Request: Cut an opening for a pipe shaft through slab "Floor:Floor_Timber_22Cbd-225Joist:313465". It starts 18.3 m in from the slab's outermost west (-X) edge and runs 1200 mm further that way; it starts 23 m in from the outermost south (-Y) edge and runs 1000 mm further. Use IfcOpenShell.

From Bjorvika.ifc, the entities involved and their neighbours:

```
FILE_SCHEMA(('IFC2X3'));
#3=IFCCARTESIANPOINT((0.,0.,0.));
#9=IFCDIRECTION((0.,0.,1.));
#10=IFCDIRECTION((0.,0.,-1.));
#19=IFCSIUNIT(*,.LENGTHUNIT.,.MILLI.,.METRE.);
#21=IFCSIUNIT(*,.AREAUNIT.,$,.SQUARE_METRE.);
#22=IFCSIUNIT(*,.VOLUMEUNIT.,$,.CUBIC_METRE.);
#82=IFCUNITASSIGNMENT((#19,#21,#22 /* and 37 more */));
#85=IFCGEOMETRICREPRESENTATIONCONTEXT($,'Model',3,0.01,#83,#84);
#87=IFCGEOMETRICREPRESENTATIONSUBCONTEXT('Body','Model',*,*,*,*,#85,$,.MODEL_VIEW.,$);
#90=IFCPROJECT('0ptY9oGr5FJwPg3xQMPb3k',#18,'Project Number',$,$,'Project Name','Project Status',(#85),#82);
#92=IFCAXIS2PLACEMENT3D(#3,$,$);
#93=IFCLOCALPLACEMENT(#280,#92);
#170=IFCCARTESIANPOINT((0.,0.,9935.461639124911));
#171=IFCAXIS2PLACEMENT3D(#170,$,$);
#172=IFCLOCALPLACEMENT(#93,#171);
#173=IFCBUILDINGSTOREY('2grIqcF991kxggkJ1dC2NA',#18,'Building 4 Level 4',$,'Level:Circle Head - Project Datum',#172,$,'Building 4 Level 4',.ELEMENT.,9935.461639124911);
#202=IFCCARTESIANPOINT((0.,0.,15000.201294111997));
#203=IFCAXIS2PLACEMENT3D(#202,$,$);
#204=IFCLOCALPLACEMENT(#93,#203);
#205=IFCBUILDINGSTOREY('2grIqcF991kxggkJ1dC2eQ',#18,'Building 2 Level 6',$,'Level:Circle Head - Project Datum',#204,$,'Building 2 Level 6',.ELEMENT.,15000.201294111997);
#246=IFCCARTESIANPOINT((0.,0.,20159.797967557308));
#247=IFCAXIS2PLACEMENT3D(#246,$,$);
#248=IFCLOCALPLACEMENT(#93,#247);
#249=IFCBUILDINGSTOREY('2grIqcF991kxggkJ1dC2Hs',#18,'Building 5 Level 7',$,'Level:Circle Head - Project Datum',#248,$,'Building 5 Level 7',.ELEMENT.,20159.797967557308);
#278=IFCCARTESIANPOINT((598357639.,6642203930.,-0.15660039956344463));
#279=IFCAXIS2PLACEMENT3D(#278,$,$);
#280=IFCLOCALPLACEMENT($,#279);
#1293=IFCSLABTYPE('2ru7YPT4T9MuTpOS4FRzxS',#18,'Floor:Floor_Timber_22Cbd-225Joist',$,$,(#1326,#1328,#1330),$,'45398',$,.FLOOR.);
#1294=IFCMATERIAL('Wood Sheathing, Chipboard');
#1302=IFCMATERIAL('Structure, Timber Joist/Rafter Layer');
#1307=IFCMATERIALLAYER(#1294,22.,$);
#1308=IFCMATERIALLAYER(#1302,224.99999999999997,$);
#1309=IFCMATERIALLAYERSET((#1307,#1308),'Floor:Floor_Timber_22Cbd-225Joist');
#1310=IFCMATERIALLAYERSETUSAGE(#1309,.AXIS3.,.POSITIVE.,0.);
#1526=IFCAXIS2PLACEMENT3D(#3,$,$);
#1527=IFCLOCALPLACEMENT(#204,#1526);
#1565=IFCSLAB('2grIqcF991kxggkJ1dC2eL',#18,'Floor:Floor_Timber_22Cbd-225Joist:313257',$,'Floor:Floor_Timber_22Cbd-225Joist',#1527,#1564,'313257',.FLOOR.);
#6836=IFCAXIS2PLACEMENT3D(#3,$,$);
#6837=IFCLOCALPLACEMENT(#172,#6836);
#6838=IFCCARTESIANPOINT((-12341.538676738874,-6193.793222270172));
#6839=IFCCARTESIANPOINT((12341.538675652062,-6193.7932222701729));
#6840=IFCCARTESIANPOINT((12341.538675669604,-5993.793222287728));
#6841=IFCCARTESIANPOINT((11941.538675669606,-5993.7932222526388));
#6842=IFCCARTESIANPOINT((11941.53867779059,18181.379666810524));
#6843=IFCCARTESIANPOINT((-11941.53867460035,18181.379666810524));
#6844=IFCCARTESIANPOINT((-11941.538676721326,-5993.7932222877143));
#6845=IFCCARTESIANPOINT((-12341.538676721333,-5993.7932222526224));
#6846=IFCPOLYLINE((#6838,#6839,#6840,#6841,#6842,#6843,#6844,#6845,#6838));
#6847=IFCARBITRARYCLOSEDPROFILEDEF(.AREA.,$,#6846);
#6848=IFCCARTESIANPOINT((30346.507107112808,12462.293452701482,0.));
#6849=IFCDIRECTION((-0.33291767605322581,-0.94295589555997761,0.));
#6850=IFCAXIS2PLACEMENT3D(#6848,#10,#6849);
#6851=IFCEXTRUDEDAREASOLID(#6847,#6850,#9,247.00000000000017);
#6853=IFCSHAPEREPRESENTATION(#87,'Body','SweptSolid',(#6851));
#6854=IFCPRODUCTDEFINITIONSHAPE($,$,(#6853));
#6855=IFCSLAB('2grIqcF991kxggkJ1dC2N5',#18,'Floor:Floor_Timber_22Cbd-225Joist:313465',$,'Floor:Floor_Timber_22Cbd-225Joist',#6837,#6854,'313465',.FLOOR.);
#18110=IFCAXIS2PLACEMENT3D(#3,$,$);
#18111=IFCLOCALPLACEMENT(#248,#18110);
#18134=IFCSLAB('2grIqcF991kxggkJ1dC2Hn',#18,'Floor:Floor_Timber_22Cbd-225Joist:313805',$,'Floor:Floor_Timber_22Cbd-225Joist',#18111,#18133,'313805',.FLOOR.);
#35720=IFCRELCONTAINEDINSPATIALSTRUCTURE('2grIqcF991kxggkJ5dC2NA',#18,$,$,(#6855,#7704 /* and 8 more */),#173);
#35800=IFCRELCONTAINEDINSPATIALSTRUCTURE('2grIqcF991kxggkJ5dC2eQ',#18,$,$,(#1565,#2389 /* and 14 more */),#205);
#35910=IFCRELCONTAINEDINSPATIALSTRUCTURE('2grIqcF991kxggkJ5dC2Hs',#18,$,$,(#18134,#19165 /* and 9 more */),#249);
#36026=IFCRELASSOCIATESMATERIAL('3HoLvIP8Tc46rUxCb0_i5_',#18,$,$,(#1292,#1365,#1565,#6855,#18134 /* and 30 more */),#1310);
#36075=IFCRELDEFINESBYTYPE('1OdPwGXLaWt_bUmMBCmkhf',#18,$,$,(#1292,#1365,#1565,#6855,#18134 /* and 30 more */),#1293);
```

```python
import numpy as np
import ifcopenshell
import ifcopenshell.api.feature
import ifcopenshell.api.geometry
import ifcopenshell.api.root
import ifcopenshell.geom
import ifcopenshell.util.placement
import ifcopenshell.util.representation
import ifcopenshell.util.shape
import ifcopenshell.util.unit

model = ifcopenshell.open("Bjorvika.ifc")
unit_scale = ifcopenshell.util.unit.calculate_unit_scale(model)
settings = ifcopenshell.geom.settings()


def volume(element):
    """Net volume in cubic metres, openings subtracted."""
    shape = ifcopenshell.geom.create_shape(settings, element)
    return ifcopenshell.util.shape.get_volume(shape.geometry)


slab = model.by_guid("2grIqcF991kxggkJ1dC2N5")
before = volume(slab)

# Extent in the slab's own axes, in metres. The edges named are its -X and -Y sides.
slab_shape = ifcopenshell.geom.create_shape(settings, slab)
vertices = ifcopenshell.util.shape.get_vertices(slab_shape.geometry)
x_min, y_min, bottom = vertices.min(axis=0)
top = vertices[:, 2].max()

opening = ifcopenshell.api.root.create_entity(model, ifc_class="IfcOpeningElement", name="Pipe shaft opening")
context = ifcopenshell.util.representation.get_context(model, "Model", "Body", "MODEL_VIEW")
width, depth = 1.2, 1
outline = [(0.0, 0.0), (width, 0.0), (width, depth), (0.0, depth), (0.0, 0.0)]
# Overshoot both faces by 50 mm so the cut is clean.
shape = ifcopenshell.api.geometry.add_slab_representation(
    model, context=context, depth=top - bottom + 0.1, polyline=outline
)
ifcopenshell.api.geometry.assign_representation(model, product=opening, representation=shape)

matrix = ifcopenshell.util.placement.get_local_placement(slab.ObjectPlacement)
matrix[:, 3] = matrix @ np.append(np.array([x_min + 18.3, y_min + 23, bottom - 0.05]) / unit_scale, 1.0)
ifcopenshell.api.geometry.edit_object_placement(model, product=opening, matrix=matrix, is_si=False)
ifcopenshell.api.feature.add_feature(model, feature=opening, element=slab)

after = volume(slab)

print(f"slab volume {before:.3f} -> {after:.3f} m3")

model.write("Bjorvika_v2.ifc")
```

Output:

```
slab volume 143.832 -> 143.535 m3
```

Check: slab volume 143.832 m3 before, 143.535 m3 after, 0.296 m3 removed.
